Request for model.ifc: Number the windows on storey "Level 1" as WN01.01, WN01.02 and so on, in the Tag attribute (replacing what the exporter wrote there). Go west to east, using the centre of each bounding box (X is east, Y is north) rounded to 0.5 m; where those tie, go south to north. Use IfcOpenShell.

First a look at what the model holds.

```python
import ifcopenshell
import ifcopenshell.util.element
import ifcopenshell.util.placement

model = ifcopenshell.open("model.ifc")
print(model.schema)
storey = next(s for s in model.by_type("IfcBuildingStorey") if s.Name == "Level 1")
windows = [e for e in ifcopenshell.util.element.get_decomposition(storey) if e.is_a("IfcWindow")]
for e in sorted(windows, key=lambda e: e.id()):
    origin = ifcopenshell.util.placement.get_local_placement(e.ObjectPlacement)[:3, 3]
    print(e.id(), e.Tag, e.Name, origin.round(2) + 0.0, sep=" | ")
```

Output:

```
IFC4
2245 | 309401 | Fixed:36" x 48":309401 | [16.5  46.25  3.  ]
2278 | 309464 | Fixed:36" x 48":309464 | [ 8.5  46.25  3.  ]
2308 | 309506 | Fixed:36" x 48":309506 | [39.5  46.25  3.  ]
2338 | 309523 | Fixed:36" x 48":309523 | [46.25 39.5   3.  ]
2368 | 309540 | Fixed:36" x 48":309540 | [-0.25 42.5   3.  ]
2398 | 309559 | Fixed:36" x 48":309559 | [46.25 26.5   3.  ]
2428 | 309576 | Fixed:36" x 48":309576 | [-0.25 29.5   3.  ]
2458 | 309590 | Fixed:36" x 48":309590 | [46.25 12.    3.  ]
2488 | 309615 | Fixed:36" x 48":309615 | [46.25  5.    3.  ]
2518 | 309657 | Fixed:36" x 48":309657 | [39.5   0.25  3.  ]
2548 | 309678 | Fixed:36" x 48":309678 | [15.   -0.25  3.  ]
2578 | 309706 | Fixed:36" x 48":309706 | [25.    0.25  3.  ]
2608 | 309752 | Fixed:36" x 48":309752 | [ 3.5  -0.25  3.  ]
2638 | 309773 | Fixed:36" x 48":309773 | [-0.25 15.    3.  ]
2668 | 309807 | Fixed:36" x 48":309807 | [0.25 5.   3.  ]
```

```python
import ifcopenshell
import ifcopenshell.geom
import ifcopenshell.util.element
import ifcopenshell.util.shape

model = ifcopenshell.open("model.ifc")
settings = ifcopenshell.geom.settings()
settings.set("use-world-coords", True)


def centre(element):
    shape = ifcopenshell.geom.create_shape(settings, element)
    return ifcopenshell.util.shape.get_bbox_centroid(shape.geometry)


storey = next(s for s in model.by_type("IfcBuildingStorey") if s.Name == "Level 1")
windows = [e for e in ifcopenshell.util.element.get_decomposition(storey) if e.is_a("IfcWindow")]

# Insertion points can sit at a corner or the storey origin, so sort by the geometry (in metres).
centres = {e: centre(e) for e in windows}
windows.sort(key=lambda e: (round(centres[e][0] / 0.5), centres[e][1]))

for i, e in enumerate(windows, start=1):
    number = f"WN01.{i:02d}"
    e.Tag = number
    print(e.id(), number)

model.write("model_updated.ifc")
```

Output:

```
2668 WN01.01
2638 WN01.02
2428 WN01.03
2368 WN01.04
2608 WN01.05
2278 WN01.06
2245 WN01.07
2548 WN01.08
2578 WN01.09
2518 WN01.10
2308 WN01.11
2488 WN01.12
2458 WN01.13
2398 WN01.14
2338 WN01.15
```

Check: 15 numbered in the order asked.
